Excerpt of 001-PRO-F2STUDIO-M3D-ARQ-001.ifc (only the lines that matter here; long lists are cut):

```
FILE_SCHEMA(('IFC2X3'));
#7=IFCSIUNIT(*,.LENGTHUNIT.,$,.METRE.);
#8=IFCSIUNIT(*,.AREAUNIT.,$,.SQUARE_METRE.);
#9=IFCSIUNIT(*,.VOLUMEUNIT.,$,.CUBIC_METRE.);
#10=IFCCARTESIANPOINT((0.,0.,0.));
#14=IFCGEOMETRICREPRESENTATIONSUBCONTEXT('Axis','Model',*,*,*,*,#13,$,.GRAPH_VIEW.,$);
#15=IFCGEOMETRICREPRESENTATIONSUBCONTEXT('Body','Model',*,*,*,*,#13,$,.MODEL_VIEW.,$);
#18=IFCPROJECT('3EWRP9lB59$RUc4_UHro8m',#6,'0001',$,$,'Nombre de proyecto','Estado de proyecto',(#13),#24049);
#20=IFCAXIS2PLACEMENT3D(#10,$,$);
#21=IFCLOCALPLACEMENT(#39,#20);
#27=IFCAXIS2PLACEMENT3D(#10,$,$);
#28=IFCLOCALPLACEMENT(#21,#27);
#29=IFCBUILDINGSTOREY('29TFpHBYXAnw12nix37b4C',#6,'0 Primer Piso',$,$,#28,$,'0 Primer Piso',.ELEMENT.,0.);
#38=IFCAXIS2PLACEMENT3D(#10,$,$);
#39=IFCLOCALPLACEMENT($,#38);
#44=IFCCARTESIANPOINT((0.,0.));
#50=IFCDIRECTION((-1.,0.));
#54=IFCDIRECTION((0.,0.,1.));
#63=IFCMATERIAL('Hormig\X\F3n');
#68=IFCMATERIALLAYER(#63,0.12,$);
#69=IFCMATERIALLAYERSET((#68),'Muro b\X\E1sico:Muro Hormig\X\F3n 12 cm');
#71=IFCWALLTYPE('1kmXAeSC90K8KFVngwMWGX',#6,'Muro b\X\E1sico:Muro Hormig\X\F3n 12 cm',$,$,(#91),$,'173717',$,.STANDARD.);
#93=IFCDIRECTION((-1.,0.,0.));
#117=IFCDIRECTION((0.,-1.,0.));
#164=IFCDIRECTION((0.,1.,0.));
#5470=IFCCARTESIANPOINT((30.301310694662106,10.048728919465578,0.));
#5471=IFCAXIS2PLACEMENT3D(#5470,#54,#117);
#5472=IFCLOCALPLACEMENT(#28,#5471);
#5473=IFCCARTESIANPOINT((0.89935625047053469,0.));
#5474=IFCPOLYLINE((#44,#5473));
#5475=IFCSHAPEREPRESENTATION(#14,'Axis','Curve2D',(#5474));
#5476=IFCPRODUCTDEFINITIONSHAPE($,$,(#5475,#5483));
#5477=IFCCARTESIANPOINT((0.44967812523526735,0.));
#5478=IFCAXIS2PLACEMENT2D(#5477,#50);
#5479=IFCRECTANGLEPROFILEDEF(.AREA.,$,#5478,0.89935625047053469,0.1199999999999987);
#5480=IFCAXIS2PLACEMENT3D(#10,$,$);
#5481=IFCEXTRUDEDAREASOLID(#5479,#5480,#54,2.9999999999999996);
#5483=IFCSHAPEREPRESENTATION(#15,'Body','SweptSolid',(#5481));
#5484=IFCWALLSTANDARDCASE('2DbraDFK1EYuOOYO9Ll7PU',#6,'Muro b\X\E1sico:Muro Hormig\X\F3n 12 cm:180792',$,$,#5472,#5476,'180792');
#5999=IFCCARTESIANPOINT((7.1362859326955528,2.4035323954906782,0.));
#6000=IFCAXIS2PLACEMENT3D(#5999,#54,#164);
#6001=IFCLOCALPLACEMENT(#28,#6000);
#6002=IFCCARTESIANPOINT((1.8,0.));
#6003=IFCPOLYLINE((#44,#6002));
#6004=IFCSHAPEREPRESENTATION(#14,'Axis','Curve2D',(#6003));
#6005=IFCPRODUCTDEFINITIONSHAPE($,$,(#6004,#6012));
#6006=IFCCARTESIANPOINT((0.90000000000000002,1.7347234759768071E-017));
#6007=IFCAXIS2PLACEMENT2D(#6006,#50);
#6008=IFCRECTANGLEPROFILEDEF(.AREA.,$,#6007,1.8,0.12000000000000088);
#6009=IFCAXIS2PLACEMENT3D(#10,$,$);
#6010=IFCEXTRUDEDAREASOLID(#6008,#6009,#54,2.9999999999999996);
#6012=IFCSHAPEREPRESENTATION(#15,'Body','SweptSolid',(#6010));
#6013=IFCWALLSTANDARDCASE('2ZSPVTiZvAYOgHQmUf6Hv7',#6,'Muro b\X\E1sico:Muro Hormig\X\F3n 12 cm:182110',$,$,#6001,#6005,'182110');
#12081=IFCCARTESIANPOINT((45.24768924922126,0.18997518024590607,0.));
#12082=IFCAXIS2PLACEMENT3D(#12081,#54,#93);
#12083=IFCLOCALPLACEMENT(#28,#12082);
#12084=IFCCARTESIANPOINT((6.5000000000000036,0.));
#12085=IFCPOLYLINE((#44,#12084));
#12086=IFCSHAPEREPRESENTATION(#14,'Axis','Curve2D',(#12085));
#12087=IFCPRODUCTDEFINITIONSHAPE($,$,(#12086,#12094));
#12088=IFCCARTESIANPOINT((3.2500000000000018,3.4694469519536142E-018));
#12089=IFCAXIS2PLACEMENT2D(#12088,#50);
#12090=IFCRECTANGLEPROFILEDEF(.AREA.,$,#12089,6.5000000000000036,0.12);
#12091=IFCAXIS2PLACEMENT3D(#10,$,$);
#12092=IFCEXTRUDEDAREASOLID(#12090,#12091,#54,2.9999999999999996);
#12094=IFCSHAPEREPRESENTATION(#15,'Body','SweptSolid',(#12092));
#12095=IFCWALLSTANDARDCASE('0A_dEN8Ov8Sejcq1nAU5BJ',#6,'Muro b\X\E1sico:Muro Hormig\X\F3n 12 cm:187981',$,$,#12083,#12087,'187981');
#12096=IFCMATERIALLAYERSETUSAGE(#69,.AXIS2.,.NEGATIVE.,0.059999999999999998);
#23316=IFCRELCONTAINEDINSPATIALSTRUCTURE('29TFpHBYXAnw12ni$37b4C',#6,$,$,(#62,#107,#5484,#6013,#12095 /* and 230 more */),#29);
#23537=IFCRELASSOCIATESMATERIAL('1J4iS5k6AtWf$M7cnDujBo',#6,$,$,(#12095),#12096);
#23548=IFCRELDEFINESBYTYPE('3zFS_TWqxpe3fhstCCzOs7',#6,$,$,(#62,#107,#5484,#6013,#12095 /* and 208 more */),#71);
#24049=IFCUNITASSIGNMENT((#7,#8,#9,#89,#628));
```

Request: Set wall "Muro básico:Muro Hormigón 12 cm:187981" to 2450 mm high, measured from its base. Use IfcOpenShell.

```python
import ifcopenshell
import ifcopenshell.geom
import ifcopenshell.util.representation
import ifcopenshell.util.shape
import ifcopenshell.util.unit

model = ifcopenshell.open("001-PRO-F2STUDIO-M3D-ARQ-001.ifc")
unit_scale = ifcopenshell.util.unit.calculate_unit_scale(model)
settings = ifcopenshell.geom.settings()


def volume(element):
    """Net volume in cubic metres, openings subtracted."""
    shape = ifcopenshell.geom.create_shape(settings, element)
    return ifcopenshell.util.shape.get_volume(shape.geometry)


wall = model.by_id(12095)
before = volume(wall)

body = ifcopenshell.util.representation.get_representation(wall, "Model", "Body")
solid = body.Items[0]
old_height = solid.Depth
solid.Depth = 2.45 / unit_scale
after = volume(wall)

print(f"height {old_height:g} -> {solid.Depth:g}, volume {before:.3f} -> {after:.3f} m3")

model.write("001-PRO-F2STUDIO-M3D-ARQ-001-out.ifc")
```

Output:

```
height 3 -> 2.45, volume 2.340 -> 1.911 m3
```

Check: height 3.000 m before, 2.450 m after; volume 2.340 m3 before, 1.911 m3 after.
